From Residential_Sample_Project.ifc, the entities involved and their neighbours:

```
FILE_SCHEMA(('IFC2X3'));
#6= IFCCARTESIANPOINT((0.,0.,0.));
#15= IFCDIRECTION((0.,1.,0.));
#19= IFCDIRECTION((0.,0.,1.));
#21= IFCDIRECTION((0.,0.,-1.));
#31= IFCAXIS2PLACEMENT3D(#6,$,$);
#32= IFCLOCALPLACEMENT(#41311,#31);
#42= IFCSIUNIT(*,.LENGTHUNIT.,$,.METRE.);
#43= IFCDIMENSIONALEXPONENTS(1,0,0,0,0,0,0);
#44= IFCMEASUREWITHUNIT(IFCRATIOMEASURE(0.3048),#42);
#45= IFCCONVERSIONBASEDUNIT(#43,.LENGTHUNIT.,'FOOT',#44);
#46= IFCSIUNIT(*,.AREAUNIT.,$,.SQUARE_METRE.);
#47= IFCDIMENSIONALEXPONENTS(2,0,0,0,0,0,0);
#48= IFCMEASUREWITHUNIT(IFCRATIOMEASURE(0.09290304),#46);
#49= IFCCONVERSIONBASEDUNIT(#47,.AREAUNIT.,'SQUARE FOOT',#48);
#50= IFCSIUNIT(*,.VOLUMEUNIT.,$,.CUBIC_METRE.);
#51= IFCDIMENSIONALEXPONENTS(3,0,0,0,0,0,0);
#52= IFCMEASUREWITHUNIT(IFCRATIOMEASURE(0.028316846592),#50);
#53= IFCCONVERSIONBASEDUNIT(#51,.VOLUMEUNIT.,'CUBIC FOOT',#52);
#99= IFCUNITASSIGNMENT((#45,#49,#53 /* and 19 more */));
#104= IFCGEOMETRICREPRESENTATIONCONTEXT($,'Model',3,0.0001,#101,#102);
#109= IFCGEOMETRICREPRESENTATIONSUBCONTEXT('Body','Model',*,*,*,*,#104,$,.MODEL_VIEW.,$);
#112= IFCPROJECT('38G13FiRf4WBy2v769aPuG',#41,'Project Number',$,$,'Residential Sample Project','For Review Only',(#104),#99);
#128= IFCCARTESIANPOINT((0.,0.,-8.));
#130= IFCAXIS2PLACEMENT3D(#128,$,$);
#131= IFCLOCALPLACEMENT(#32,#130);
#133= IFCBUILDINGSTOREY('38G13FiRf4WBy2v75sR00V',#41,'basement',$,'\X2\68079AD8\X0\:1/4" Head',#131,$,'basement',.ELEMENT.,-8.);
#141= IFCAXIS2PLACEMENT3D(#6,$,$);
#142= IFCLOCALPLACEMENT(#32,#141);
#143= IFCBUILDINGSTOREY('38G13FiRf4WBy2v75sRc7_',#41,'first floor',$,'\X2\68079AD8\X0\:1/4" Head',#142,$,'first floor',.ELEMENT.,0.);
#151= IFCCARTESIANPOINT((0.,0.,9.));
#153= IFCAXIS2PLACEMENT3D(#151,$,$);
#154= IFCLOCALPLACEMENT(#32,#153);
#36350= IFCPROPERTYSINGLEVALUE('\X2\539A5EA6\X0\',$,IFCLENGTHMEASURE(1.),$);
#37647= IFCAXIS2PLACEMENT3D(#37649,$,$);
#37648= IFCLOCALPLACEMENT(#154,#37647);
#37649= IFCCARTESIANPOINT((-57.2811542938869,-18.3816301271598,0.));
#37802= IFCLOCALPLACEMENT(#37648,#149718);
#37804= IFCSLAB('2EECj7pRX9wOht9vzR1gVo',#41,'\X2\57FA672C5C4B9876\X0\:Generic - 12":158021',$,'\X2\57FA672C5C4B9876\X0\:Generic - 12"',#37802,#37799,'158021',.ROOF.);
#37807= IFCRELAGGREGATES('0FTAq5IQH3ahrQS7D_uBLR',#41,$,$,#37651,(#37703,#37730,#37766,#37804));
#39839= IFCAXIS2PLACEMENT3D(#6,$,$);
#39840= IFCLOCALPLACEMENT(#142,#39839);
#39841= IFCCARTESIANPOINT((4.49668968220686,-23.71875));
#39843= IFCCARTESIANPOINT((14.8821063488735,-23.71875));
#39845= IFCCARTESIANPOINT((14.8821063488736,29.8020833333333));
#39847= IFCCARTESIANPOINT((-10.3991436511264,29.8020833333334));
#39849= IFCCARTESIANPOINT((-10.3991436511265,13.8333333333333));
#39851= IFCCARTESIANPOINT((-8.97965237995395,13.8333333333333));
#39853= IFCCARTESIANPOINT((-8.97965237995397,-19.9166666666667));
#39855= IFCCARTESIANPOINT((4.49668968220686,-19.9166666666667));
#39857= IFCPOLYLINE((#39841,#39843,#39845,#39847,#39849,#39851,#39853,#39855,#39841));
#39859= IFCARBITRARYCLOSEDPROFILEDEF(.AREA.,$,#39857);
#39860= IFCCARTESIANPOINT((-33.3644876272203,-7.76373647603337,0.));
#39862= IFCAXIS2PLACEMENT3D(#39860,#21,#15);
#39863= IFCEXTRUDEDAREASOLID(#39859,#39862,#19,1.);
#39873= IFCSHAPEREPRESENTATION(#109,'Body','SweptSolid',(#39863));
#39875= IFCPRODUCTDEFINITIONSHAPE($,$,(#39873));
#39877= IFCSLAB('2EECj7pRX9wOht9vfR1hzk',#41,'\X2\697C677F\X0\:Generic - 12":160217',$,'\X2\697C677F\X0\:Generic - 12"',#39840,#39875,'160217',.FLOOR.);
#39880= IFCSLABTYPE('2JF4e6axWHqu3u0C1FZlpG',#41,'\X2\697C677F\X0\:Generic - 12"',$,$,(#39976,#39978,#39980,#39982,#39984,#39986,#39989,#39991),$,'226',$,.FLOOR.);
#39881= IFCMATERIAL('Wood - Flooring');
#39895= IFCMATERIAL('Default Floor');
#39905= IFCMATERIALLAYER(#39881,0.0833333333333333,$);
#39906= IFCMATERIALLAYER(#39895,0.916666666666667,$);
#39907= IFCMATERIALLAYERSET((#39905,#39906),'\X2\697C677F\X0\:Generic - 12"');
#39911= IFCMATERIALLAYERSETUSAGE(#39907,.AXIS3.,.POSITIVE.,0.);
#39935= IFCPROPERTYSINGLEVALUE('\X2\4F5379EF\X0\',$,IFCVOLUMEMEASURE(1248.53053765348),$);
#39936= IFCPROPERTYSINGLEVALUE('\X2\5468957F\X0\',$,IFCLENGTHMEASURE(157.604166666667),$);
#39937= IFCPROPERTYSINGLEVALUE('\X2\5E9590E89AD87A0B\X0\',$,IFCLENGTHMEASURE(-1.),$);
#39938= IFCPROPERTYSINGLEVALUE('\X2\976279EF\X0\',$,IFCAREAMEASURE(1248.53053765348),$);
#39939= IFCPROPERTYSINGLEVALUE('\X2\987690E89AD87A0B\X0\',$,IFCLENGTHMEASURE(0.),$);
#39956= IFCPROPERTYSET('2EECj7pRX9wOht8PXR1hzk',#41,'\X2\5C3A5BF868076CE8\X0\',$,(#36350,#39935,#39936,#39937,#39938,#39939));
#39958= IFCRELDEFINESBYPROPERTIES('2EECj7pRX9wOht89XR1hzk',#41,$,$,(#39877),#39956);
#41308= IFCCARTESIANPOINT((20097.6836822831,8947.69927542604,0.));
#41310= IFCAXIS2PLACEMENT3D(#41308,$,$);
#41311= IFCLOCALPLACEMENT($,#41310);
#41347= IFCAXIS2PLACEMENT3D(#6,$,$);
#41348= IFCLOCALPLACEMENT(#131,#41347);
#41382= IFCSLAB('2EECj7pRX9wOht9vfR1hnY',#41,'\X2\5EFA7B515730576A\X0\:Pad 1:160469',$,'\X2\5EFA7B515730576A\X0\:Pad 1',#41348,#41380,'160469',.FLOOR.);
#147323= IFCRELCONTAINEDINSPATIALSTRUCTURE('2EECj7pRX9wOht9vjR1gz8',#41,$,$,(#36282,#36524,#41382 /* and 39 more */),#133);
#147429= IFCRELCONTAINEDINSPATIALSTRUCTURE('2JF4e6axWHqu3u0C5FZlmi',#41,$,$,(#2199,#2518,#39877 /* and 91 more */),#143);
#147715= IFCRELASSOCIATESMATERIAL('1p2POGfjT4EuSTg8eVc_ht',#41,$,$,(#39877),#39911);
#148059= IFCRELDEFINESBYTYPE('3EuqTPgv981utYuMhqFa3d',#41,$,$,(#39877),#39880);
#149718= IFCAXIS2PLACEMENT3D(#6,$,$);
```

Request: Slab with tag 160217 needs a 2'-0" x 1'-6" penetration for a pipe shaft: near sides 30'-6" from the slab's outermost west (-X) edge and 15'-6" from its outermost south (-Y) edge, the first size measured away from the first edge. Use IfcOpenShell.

```python
import numpy as np
import ifcopenshell
import ifcopenshell.api.feature
import ifcopenshell.api.geometry
import ifcopenshell.api.pset
import ifcopenshell.api.root
import ifcopenshell.geom
import ifcopenshell.util.element
import ifcopenshell.util.placement
import ifcopenshell.util.representation
import ifcopenshell.util.shape
import ifcopenshell.util.unit

model = ifcopenshell.open("Residential_Sample_Project.ifc")
unit_scale = ifcopenshell.util.unit.calculate_unit_scale(model)
area_scale = ifcopenshell.util.unit.calculate_unit_scale(model, "AREAUNIT")
volume_scale = ifcopenshell.util.unit.calculate_unit_scale(model, "VOLUMEUNIT")
settings = ifcopenshell.geom.settings()


def volume(element):
    """Net volume in cubic metres, openings subtracted."""
    shape = ifcopenshell.geom.create_shape(settings, element)
    return ifcopenshell.util.shape.get_volume(shape.geometry)


slab = model.by_guid("2EECj7pRX9wOht9vfR1hzk")
before = volume(slab)

# Extent in the slab's own axes, in metres. The edges named are its -X and -Y sides.
slab_shape = ifcopenshell.geom.create_shape(settings, slab)
vertices = ifcopenshell.util.shape.get_vertices(slab_shape.geometry)
x_min, y_min, bottom = vertices.min(axis=0)
top = vertices[:, 2].max()

opening = ifcopenshell.api.root.create_entity(model, ifc_class="IfcOpeningElement", name="Pipe shaft opening")
context = ifcopenshell.util.representation.get_context(model, "Model", "Body", "MODEL_VIEW")
width, depth = 0.6096, 0.4572
outline = [(0.0, 0.0), (width, 0.0), (width, depth), (0.0, depth), (0.0, 0.0)]
# Overshoot both faces by 50 mm so the cut is clean.
shape = ifcopenshell.api.geometry.add_slab_representation(
    model, context=context, depth=top - bottom + 0.1, polyline=outline
)
ifcopenshell.api.geometry.assign_representation(model, product=opening, representation=shape)

matrix = ifcopenshell.util.placement.get_local_placement(slab.ObjectPlacement)
matrix[:, 3] = matrix @ np.append(np.array([x_min + 9.2964, y_min + 4.7244, bottom - 0.05]) / unit_scale, 1.0)
ifcopenshell.api.geometry.edit_object_placement(model, product=opening, matrix=matrix, is_si=False)
ifcopenshell.api.feature.add_feature(model, feature=opening, element=slab)

after = volume(slab)

# Update the slab's stored quantities.
pset = model.by_id(ifcopenshell.util.element.get_pset(slab, "尺寸标注", should_inherit=False)["id"])
ifcopenshell.api.pset.edit_pset(model, pset=pset, properties={
    "体积": model.create_entity("IfcVolumeMeasure", after / volume_scale),
    "面积": model.create_entity("IfcAreaMeasure", after / (top - bottom) / area_scale),
})

print(f"slab volume {before:.3f} -> {after:.3f} m3")

model.write("Residential_Sample_Project-out.ifc")
```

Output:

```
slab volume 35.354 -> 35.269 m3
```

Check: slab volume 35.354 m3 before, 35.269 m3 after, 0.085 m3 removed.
